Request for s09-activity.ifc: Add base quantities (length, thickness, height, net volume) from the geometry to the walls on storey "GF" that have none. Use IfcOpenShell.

First a look at what the model holds.

```python
import ifcopenshell
import ifcopenshell.util.element
import ifcopenshell.util.unit

model = ifcopenshell.open("s09-activity.ifc")
print(model.schema)
for unit_type in ("LENGTHUNIT", "AREAUNIT", "VOLUMEUNIT"):
    print(unit_type, ifcopenshell.util.unit.calculate_unit_scale(model, unit_type))
storey = next(s for s in model.by_type("IfcBuildingStorey") if s.Name == "GF")
walls = [e for e in ifcopenshell.util.element.get_decomposition(storey) if e.is_a("IfcWall")]
for e in sorted(walls, key=lambda e: e.id()):
    print(e.id(), e.is_a(), e.Name, list(ifcopenshell.util.element.get_psets(e, qtos_only=True)), sep=" | ")
```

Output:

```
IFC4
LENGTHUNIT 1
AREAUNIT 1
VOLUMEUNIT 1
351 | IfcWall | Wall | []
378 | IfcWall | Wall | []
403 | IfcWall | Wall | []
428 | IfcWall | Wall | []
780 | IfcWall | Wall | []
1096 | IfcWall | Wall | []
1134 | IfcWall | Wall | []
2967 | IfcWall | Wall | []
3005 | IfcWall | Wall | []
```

```python
import ifcopenshell
import ifcopenshell.api.pset
import ifcopenshell.geom
import ifcopenshell.util.element
import ifcopenshell.util.shape
import ifcopenshell.util.unit

model = ifcopenshell.open("s09-activity.ifc")
unit_scale = ifcopenshell.util.unit.calculate_unit_scale(model)
volume_scale = ifcopenshell.util.unit.calculate_unit_scale(model, "VOLUMEUNIT")
settings = ifcopenshell.geom.settings()

storey = next(s for s in model.by_type("IfcBuildingStorey") if s.Name == "GF")
walls = [e for e in ifcopenshell.util.element.get_decomposition(storey) if e.is_a("IfcWall")]

for e in sorted(walls, key=lambda e: e.id()):
    if ifcopenshell.util.element.get_psets(e, qtos_only=True, should_inherit=False):
        continue
    # Geometry comes back in metres, in the element's own axes.
    shape = ifcopenshell.geom.create_shape(settings, e)
    values = {
        "Length": ifcopenshell.util.shape.get_x(shape.geometry) / unit_scale,
        "Width": ifcopenshell.util.shape.get_y(shape.geometry) / unit_scale,
        "Height": ifcopenshell.util.shape.get_z(shape.geometry) / unit_scale,
        "NetVolume": ifcopenshell.util.shape.get_volume(shape.geometry) / volume_scale,
    }
    qto = ifcopenshell.api.pset.add_qto(model, product=e, name="Qto_WallBaseQuantities")
    ifcopenshell.api.pset.edit_qto(model, qto=qto, properties=values)
    print(e.id(), {k: round(v, 3) for k, v in values.items()})

model.write("s09-activity_v2.ifc")
```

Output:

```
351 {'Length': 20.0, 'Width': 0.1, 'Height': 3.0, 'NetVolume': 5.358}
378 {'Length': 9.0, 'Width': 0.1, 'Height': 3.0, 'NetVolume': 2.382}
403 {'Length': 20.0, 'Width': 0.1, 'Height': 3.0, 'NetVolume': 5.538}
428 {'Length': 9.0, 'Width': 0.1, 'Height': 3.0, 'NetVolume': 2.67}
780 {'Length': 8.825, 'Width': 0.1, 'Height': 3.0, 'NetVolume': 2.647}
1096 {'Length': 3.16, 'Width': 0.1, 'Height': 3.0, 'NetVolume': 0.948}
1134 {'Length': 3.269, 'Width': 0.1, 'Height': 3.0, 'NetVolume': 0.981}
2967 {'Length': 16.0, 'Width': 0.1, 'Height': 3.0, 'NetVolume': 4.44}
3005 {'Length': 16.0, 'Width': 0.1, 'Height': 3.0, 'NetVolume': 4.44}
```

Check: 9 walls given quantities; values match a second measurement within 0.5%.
